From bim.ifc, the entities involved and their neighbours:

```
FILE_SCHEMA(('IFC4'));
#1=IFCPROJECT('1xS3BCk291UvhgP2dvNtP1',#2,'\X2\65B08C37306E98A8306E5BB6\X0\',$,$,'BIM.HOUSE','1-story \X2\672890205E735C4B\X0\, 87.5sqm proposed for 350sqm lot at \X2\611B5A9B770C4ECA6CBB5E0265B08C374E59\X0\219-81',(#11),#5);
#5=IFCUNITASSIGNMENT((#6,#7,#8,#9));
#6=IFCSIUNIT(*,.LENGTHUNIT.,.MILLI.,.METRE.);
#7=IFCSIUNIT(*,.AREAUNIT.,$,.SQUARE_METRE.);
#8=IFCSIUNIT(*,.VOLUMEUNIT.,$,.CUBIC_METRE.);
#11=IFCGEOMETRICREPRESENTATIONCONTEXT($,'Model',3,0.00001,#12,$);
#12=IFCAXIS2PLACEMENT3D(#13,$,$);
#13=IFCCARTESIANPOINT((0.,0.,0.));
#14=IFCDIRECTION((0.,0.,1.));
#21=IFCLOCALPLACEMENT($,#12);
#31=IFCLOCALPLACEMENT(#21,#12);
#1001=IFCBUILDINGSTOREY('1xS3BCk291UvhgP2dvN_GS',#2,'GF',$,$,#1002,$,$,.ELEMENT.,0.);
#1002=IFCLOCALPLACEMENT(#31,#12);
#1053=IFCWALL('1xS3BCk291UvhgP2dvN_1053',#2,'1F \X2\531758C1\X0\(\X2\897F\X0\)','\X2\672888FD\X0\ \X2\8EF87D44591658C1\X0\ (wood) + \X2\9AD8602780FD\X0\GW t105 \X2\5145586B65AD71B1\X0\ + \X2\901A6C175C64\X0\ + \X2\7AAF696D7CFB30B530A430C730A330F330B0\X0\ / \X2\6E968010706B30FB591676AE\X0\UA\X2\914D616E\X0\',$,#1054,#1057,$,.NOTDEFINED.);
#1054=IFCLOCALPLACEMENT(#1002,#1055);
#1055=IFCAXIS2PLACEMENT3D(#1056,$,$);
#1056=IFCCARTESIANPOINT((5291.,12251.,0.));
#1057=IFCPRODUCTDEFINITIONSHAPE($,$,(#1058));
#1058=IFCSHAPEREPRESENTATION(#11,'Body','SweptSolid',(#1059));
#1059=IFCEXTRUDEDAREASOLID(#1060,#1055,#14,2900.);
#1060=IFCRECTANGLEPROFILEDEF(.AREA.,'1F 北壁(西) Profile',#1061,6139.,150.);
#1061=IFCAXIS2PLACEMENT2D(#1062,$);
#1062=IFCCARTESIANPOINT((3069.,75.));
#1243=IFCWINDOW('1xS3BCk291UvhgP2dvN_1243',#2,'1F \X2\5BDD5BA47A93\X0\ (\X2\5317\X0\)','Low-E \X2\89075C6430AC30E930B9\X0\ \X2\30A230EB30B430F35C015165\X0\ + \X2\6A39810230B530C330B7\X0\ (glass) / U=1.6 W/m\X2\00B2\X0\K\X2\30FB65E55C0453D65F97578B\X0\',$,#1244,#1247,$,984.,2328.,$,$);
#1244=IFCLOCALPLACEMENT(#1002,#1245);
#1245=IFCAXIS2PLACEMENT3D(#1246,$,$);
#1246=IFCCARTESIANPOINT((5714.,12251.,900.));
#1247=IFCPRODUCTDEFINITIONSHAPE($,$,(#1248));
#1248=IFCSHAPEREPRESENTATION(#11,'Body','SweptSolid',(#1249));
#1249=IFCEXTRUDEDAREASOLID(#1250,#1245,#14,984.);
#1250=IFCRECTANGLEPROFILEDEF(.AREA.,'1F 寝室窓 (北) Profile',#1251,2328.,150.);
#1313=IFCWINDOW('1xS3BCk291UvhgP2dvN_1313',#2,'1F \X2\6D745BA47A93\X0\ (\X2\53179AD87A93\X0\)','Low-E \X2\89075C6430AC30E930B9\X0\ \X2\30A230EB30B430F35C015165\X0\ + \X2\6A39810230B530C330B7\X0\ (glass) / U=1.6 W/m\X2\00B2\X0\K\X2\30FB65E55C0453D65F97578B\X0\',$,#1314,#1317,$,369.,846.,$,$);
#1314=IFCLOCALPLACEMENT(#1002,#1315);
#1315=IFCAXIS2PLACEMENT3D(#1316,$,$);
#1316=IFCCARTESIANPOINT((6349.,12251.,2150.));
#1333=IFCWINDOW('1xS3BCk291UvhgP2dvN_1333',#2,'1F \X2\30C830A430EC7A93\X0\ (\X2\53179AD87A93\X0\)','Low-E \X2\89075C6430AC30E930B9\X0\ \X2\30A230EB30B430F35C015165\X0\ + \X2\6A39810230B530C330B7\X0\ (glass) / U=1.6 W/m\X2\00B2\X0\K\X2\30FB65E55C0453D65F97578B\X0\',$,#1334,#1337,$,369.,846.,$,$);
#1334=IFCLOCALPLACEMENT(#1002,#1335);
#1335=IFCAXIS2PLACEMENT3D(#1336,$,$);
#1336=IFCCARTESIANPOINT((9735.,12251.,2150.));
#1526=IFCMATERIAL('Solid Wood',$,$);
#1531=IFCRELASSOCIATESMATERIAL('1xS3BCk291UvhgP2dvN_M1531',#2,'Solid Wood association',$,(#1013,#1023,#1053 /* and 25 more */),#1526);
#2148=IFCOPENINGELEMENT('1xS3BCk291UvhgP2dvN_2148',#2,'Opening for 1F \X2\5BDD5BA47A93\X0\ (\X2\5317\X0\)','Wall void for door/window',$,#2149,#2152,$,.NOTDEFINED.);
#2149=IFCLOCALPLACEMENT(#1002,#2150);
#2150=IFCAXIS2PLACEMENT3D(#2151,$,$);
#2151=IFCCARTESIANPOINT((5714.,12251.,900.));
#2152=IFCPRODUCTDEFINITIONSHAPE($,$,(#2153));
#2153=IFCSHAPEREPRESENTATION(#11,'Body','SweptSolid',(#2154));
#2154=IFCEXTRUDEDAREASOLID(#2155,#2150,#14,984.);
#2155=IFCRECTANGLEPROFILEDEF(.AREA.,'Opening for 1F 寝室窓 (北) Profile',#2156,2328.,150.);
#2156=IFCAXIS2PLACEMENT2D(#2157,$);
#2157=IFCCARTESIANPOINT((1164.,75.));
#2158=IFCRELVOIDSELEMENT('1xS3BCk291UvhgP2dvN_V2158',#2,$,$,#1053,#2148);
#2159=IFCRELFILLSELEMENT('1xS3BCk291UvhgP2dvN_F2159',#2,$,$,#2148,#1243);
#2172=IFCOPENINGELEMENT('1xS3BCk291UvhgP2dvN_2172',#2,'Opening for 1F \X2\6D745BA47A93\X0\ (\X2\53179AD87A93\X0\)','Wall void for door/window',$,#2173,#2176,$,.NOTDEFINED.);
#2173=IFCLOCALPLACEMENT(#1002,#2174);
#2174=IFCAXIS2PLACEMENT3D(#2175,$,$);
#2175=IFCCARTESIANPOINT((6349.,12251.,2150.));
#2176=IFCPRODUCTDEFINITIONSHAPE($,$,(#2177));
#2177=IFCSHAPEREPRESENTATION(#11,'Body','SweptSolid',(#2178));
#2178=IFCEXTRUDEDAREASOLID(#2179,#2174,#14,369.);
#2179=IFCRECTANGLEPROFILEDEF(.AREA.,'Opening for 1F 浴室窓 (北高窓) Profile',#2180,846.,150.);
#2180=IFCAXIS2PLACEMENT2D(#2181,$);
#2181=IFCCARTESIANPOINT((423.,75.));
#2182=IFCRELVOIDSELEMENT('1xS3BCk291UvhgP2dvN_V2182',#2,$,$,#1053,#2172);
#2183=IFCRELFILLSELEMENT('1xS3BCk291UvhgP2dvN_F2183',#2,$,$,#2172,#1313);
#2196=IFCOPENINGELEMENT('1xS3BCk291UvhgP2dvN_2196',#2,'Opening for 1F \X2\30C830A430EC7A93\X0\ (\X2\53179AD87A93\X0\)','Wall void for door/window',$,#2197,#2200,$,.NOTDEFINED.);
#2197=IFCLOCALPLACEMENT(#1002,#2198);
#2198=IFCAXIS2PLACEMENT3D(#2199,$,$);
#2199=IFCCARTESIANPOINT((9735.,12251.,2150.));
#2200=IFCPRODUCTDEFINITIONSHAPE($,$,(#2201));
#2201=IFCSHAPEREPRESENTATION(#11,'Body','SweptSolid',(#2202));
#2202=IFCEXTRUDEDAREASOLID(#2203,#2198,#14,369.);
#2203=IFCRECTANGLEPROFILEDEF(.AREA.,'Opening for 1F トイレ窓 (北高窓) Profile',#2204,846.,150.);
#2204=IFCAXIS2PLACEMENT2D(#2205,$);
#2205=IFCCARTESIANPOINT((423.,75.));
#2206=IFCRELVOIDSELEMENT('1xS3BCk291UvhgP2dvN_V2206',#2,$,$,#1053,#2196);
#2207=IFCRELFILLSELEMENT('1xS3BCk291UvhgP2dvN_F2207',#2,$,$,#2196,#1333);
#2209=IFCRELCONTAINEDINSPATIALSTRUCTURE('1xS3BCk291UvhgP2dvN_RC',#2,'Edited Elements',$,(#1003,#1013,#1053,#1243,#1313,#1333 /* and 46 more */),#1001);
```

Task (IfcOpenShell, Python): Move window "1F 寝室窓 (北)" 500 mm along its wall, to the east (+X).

```python
import ifcopenshell
import ifcopenshell.api.geometry
import ifcopenshell.util.placement
import ifcopenshell.util.unit

model = ifcopenshell.open("bim.ifc")
unit_scale = ifcopenshell.util.unit.calculate_unit_scale(model)

window = model.by_guid("1xS3BCk291UvhgP2dvN_1243")
opening = window.FillsVoids[0].RelatingOpeningElement
wall = opening.VoidsElements[0].RelatingBuildingElement

wall_matrix = ifcopenshell.util.placement.get_local_placement(wall.ObjectPlacement)
shift = wall_matrix[:3, 0] * 0.5 / unit_scale
before = ifcopenshell.util.placement.get_local_placement(window.ObjectPlacement)[:3, 3].copy()

# The window is not placed relative to its opening, so move both.
for product in (opening, window):
    matrix = ifcopenshell.util.placement.get_local_placement(product.ObjectPlacement)
    matrix[:3, 3] += shift
    ifcopenshell.api.geometry.edit_object_placement(model, product=product, matrix=matrix, is_si=False)

after = ifcopenshell.util.placement.get_local_placement(window.ObjectPlacement)[:3, 3]
print("window moved by", (after - before).round(3) + 0.0)

model.write("bim_rev.ifc")
```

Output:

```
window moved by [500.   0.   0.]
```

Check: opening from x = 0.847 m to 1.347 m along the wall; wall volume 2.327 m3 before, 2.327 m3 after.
